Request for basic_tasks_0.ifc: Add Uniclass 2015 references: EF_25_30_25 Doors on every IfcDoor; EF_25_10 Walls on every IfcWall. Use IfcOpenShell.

First a look at what the model holds.

```python
import ifcopenshell

model = ifcopenshell.open("basic_tasks_0.ifc")
print(model.schema)
print("classifications:", [c.Name for c in model.by_type("IfcClassification")])
for ifc_class in ("IfcDoor", "IfcRoof", "IfcStair", "IfcWall", "IfcWindow"):
    print(ifc_class, len(model.by_type(ifc_class)))
```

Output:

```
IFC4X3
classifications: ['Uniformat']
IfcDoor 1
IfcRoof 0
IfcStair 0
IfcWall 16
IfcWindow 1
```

```python
import ifcopenshell
import ifcopenshell.api.classification

model = ifcopenshell.open("basic_tasks_0.ifc")

system = ifcopenshell.api.classification.add_classification(model, classification="Uniclass 2015")

codes = {
    "IfcDoor": ("EF_25_30_25", "Doors"),
    "IfcWall": ("EF_25_10", "Walls"),
}
for ifc_class, (code, name) in codes.items():
    products = model.by_type(ifc_class)
    ifcopenshell.api.classification.add_reference(
        model, products=products, classification=system, identification=code, name=name
    )
    print(code, len(products))

model.write("basic_tasks_0_updated.ifc")
```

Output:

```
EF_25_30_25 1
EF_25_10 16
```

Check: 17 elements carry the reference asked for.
